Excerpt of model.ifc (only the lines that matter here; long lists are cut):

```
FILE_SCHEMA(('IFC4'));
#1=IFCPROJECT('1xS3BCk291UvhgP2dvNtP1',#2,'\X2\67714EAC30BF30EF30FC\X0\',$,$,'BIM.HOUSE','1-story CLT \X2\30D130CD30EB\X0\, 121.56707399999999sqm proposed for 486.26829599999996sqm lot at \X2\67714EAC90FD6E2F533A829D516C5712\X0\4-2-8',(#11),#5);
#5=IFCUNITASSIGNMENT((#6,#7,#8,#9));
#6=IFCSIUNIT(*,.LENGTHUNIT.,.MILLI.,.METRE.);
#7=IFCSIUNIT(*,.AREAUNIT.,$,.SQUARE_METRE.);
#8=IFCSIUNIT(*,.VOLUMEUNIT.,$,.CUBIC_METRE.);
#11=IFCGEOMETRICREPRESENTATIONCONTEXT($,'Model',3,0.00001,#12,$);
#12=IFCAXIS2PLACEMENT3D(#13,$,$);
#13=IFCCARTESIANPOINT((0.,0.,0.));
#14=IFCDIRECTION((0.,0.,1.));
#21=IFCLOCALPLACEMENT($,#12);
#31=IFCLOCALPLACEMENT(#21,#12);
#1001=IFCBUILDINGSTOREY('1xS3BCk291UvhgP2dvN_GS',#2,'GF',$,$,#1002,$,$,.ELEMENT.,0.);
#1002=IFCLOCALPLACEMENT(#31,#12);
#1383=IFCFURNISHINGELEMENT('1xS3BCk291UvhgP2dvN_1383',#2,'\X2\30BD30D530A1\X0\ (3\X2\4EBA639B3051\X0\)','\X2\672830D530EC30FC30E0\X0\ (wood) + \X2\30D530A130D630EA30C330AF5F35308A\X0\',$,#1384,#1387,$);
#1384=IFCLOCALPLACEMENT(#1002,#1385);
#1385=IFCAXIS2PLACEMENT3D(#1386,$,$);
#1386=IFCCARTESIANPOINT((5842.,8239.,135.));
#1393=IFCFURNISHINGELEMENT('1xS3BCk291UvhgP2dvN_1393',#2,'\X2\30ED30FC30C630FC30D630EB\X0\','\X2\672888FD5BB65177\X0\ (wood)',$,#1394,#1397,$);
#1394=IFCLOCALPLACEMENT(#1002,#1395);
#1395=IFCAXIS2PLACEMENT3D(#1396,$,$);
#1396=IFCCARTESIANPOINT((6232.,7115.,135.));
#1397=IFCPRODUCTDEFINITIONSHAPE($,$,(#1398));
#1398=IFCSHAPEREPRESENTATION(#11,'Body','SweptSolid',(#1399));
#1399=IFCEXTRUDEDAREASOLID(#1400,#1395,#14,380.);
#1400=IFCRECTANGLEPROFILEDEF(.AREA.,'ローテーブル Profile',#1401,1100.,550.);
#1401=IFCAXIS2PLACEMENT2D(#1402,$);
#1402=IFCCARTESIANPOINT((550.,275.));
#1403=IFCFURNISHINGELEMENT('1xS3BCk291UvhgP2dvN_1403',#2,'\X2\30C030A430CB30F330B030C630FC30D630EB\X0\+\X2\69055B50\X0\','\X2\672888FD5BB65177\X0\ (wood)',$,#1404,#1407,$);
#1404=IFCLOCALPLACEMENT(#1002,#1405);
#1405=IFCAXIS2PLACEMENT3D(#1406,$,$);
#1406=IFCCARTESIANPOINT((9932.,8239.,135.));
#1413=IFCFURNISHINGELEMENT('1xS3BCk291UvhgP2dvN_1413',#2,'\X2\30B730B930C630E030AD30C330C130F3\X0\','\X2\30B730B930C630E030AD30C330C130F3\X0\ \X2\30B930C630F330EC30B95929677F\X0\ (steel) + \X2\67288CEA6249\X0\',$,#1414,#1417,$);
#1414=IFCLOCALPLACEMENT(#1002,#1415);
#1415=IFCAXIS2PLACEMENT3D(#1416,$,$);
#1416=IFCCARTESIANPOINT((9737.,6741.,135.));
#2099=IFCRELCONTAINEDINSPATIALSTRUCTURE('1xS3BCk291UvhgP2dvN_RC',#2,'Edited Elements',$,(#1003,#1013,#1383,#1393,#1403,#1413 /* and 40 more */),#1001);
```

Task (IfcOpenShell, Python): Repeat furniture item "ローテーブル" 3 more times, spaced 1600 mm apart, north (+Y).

```python
import numpy as np
import ifcopenshell
import ifcopenshell.api.geometry
import ifcopenshell.api.root
import ifcopenshell.util.element
import ifcopenshell.util.placement
import ifcopenshell.util.unit

model = ifcopenshell.open("model.ifc")
unit_scale = ifcopenshell.util.unit.calculate_unit_scale(model)


def reuse_history(source, copy):
    """copy_class also copies each property set's owner history, people and application; keep the originals."""
    for rel in copy.IsDefinedBy:
        if rel.is_a("IfcRelDefinesByProperties") and (history := rel.RelatingPropertyDefinition.OwnerHistory):
            rel.RelatingPropertyDefinition.OwnerHistory = source.OwnerHistory
            ifcopenshell.util.element.remove_deep2(model, history)


source = model.by_guid("1xS3BCk291UvhgP2dvN_1393")
base = ifcopenshell.util.placement.get_local_placement(source.ObjectPlacement)
step = np.array([0.0, 1.0, 0.0]) * 1.6 / unit_scale

for i in range(1, 4):
    copy = ifcopenshell.api.root.copy_class(model, product=source)
    copy.Representation = ifcopenshell.util.element.copy_deep(
        model, source.Representation, exclude=["IfcGeometricRepresentationContext", "IfcRepresentationMap"]
    )
    reuse_history(source, copy)
    matrix = base.copy()
    matrix[:3, 3] += i * step
    print("added at", matrix[:3, 3].round(3) + 0.0)
    ifcopenshell.api.geometry.edit_object_placement(model, product=copy, matrix=matrix, is_si=False)

model.write("model_v2.ifc")
```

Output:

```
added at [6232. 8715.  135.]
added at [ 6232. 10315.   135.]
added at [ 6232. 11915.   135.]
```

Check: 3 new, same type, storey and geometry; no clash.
